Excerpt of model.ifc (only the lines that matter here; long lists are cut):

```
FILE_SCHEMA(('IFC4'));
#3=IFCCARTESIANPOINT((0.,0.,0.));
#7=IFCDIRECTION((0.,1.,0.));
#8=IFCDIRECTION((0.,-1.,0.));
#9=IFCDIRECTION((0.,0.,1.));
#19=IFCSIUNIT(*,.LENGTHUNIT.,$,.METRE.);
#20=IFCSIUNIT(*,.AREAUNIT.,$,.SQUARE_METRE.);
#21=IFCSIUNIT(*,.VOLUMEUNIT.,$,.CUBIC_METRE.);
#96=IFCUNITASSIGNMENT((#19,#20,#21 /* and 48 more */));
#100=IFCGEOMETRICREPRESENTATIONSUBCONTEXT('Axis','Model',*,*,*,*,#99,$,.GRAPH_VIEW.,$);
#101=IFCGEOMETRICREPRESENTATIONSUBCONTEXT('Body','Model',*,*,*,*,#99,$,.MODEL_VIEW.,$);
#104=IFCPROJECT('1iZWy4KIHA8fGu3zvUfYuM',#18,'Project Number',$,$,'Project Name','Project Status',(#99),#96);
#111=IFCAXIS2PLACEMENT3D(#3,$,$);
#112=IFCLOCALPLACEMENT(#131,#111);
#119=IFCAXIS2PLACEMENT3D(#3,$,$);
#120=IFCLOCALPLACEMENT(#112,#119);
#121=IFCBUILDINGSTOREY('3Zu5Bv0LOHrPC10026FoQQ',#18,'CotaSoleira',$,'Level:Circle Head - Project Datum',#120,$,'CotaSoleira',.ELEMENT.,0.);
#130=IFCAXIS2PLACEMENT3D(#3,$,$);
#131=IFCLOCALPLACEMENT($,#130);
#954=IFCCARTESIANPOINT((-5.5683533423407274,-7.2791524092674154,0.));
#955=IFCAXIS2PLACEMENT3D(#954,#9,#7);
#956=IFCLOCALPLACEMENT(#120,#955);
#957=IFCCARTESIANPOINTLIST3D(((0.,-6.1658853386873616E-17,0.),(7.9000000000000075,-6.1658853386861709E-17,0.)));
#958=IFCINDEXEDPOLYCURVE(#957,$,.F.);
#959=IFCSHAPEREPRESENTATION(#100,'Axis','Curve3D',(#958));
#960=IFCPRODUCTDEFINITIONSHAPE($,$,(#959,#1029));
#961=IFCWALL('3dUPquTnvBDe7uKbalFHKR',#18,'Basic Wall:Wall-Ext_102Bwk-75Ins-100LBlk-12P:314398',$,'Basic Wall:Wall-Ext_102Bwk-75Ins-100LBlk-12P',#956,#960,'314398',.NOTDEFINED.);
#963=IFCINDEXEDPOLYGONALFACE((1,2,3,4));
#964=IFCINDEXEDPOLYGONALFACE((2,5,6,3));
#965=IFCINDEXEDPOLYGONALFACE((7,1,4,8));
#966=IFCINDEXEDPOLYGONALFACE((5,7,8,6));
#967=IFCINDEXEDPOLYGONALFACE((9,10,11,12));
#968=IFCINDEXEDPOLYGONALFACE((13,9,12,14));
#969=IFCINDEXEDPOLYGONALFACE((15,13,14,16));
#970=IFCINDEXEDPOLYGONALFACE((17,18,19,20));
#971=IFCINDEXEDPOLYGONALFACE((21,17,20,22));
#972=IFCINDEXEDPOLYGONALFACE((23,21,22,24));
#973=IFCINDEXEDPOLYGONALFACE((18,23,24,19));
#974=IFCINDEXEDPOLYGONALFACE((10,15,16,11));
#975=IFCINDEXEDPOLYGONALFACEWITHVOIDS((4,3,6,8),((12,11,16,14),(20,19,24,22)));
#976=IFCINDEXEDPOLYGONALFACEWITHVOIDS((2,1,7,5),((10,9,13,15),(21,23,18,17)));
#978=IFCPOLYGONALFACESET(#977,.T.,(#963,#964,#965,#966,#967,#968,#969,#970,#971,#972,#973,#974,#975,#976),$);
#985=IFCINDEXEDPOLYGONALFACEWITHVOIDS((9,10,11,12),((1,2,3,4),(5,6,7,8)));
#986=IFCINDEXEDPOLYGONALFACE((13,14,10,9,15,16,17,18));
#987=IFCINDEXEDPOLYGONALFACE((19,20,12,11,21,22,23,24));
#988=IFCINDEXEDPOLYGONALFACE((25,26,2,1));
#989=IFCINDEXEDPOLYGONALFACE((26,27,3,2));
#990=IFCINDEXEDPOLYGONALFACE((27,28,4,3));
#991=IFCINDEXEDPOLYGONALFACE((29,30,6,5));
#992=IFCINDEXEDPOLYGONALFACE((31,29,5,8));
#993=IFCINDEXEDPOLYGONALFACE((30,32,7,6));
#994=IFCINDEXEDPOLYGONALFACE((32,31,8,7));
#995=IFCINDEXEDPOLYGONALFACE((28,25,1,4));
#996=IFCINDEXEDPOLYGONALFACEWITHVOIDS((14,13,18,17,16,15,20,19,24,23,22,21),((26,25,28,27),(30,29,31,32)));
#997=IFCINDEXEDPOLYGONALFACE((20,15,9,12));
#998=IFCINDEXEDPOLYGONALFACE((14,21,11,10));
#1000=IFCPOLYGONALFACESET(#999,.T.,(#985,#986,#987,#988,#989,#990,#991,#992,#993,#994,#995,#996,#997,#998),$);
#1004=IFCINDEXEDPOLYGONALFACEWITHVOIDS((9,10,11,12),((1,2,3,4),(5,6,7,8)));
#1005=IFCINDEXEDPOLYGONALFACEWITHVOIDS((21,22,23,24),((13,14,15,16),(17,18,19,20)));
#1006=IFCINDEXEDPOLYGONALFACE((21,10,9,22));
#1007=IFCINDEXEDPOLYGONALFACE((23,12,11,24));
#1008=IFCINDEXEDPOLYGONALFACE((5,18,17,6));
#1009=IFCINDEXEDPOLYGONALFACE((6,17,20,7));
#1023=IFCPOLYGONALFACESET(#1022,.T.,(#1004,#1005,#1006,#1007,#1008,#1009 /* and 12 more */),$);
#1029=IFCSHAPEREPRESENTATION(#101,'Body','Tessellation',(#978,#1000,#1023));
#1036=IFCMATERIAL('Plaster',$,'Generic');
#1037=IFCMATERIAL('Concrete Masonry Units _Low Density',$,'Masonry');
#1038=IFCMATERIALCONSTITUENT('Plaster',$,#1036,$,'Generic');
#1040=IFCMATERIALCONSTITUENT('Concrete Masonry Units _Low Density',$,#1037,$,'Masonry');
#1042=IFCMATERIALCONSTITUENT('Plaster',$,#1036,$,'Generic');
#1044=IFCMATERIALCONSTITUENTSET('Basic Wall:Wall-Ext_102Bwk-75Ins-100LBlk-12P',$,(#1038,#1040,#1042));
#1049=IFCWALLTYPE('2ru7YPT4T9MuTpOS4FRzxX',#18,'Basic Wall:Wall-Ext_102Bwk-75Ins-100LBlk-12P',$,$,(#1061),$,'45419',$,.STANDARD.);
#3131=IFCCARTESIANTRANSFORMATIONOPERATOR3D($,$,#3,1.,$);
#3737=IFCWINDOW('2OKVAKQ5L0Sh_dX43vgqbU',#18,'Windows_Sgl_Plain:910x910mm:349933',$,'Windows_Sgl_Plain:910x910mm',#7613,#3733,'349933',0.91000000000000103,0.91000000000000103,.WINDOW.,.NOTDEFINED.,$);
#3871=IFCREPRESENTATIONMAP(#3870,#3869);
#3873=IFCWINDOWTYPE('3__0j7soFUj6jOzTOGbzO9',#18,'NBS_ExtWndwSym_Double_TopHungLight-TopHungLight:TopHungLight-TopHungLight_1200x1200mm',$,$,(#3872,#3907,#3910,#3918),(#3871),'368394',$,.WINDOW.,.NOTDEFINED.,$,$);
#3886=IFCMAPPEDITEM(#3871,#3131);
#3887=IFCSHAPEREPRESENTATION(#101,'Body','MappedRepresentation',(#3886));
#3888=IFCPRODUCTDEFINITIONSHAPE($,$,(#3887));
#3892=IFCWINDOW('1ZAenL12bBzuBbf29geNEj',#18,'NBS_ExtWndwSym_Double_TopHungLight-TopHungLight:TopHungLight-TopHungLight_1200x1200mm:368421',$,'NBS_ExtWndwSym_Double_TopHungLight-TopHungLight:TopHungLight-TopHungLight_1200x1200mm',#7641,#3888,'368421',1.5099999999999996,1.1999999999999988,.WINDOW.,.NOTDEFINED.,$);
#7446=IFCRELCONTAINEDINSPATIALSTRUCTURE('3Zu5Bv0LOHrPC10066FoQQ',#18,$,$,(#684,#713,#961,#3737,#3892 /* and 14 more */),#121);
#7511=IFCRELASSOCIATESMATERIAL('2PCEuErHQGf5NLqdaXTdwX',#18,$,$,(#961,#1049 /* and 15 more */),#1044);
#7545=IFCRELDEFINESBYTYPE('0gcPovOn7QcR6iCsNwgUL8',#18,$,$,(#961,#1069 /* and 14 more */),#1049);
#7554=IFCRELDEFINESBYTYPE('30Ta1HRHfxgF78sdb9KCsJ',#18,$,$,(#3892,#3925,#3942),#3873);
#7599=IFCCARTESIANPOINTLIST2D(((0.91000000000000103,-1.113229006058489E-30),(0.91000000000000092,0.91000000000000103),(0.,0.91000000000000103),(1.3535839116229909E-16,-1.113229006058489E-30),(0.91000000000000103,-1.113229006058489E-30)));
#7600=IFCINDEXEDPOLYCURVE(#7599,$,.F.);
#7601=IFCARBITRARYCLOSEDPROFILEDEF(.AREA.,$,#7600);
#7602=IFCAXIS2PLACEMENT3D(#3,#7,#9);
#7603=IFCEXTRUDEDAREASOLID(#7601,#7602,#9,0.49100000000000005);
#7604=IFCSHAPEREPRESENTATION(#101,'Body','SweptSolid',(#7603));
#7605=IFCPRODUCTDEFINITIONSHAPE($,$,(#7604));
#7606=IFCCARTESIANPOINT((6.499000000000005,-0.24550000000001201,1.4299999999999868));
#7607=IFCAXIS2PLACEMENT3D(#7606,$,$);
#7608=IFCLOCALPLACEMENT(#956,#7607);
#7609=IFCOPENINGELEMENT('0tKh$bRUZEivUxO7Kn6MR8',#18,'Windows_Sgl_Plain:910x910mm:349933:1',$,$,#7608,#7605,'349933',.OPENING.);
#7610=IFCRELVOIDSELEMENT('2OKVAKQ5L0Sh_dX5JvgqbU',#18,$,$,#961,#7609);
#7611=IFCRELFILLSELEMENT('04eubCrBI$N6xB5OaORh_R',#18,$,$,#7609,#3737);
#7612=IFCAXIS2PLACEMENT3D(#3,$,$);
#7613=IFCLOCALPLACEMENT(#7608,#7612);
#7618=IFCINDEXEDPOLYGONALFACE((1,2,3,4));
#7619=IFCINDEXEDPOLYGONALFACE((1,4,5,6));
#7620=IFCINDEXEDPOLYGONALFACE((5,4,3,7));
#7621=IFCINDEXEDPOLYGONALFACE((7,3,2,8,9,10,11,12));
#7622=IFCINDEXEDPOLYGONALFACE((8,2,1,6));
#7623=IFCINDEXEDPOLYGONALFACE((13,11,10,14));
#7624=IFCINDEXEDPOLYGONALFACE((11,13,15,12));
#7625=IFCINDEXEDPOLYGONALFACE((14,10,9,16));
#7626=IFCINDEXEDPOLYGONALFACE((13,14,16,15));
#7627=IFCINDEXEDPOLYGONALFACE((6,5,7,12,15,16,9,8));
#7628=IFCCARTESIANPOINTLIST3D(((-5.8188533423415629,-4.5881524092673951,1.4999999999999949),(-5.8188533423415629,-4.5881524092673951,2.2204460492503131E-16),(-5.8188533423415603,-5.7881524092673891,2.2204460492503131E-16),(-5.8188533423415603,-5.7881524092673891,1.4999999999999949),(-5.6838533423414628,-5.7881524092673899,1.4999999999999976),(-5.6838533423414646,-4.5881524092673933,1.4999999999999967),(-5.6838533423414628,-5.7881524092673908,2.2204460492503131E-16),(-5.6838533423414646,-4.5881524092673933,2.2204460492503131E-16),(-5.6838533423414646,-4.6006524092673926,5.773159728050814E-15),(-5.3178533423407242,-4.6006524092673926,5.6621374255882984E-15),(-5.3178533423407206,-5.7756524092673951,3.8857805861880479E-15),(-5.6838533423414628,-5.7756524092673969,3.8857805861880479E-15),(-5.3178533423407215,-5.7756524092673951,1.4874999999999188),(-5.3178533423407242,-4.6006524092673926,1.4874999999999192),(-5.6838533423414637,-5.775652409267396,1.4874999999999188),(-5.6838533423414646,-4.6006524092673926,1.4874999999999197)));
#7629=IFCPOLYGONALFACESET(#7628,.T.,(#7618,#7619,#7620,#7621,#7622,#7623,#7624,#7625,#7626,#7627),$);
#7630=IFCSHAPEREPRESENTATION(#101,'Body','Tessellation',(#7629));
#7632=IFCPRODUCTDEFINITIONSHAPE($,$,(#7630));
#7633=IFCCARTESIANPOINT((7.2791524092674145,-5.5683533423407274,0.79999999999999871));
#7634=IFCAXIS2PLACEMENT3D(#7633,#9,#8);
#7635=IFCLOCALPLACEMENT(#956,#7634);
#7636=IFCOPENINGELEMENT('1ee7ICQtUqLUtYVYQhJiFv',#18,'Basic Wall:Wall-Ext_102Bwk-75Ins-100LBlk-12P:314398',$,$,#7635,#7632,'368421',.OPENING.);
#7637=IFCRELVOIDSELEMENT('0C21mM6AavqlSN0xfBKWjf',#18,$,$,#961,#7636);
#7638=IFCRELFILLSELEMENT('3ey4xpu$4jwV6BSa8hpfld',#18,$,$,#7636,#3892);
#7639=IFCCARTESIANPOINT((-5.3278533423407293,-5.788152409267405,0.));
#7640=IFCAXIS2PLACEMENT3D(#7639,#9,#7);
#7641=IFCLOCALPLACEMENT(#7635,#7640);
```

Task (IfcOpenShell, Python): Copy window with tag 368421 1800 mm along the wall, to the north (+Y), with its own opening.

```python
import ifcopenshell
import ifcopenshell.api.feature
import ifcopenshell.api.geometry
import ifcopenshell.api.root
import ifcopenshell.geom
import ifcopenshell.util.element
import ifcopenshell.util.placement
import ifcopenshell.util.shape

model = ifcopenshell.open("model.ifc")
settings = ifcopenshell.geom.settings()


def volume(element):
    """Net volume in cubic metres, openings subtracted."""
    shape = ifcopenshell.geom.create_shape(settings, element)
    return ifcopenshell.util.shape.get_volume(shape.geometry)


def reuse_history(source, copy):
    """copy_class also copies each property set's owner history, people and application; keep the originals."""
    for rel in copy.IsDefinedBy:
        if rel.is_a("IfcRelDefinesByProperties") and (history := rel.RelatingPropertyDefinition.OwnerHistory):
            rel.RelatingPropertyDefinition.OwnerHistory = source.OwnerHistory
            ifcopenshell.util.element.remove_deep2(model, history)


window = model.by_guid("1ZAenL12bBzuBbf29geNEj")
opening = window.FillsVoids[0].RelatingOpeningElement
wall = opening.VoidsElements[0].RelatingBuildingElement
before = volume(wall)
shift = ifcopenshell.util.placement.get_local_placement(wall.ObjectPlacement)[:3, 0] * 1.8

# copy_class copies the void relationship, type, container and properties, but no geometry.
new_opening = ifcopenshell.api.root.copy_class(model, product=opening)
new_opening.Representation = ifcopenshell.util.element.copy_deep(
    model, opening.Representation, exclude=["IfcGeometricRepresentationContext", "IfcRepresentationMap"]
)
new_opening.Name = "Basic Wall:Wall-Ext_102Bwk-75Ins-100LBlk-12P"
new_opening.Tag = None
new_window = ifcopenshell.api.root.copy_class(model, product=window)
new_window.Representation = ifcopenshell.util.element.copy_deep(
    model, window.Representation, exclude=["IfcGeometricRepresentationContext", "IfcRepresentationMap"]
)
new_window.Name = "NBS_ExtWndwSym_Double_TopHungLight-TopHungLight:TopHungLight-TopHungLight_1200x1200mm"
new_window.Tag = None
reuse_history(window, new_window)
ifcopenshell.api.feature.add_filling(model, opening=new_opening, element=new_window)

for old, new in ((opening, new_opening), (window, new_window)):
    matrix = ifcopenshell.util.placement.get_local_placement(old.ObjectPlacement)
    matrix[:3, 3] += shift
    ifcopenshell.api.geometry.edit_object_placement(model, product=new, matrix=matrix, is_si=False)

after = volume(wall)

print(f"wall volume {before:.3f} -> {after:.3f} m3")

model.write("model_rev.ifc")
```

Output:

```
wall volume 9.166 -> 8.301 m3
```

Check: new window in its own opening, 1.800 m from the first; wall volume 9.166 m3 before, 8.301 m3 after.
